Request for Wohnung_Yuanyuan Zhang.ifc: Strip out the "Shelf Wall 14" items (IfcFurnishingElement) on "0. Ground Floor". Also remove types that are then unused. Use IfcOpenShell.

First a look at what the model holds.

```python
import ifcopenshell
import ifcopenshell.util.element

model = ifcopenshell.open("Wohnung_Yuanyuan Zhang.ifc")
print(model.schema)
storey = next(s for s in model.by_type("IfcBuildingStorey") if s.Name == "0. Ground Floor")
furniture = [e for e in ifcopenshell.util.element.get_decomposition(storey) if e.is_a("IfcFurnishingElement")]
seen = {}
for e in furniture:
    element_type = ifcopenshell.util.element.get_type(e)
    name = element_type.Name if element_type not in (None, e) else None
    seen[name] = seen.get(name, 0) + 1
for name, count in sorted(seen.items(), key=str):
    print(count, "x", name)
```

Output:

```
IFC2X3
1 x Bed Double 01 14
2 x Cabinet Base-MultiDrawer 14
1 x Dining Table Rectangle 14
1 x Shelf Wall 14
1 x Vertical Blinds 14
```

```python
import ifcopenshell
import ifcopenshell.api.root
import ifcopenshell.util.element

model = ifcopenshell.open("Wohnung_Yuanyuan Zhang.ifc")

storey = next(s for s in model.by_type("IfcBuildingStorey") if s.Name == "0. Ground Floor")
furniture = [e for e in ifcopenshell.util.element.get_decomposition(storey) if e.is_a("IfcFurnishingElement")]
targets = [e for e in furniture if (t := ifcopenshell.util.element.get_type(e)) not in (None, e) and t.Name == "Shelf Wall 14"]
types = {ifcopenshell.util.element.get_type(e) for e in targets} - {None, *targets}

for e in targets:
    ifcopenshell.api.root.remove_product(model, product=e)
print(len(targets), "removed")

unused = [t for t in types if not ifcopenshell.util.element.get_types(t)]
for t in unused:
    ifcopenshell.api.root.remove_product(model, product=t)
print(len(unused), "unused types removed")

model.write("Wohnung_Yuanyuan Zhang_v2.ifc")
```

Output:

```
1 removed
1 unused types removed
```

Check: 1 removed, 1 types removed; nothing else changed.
